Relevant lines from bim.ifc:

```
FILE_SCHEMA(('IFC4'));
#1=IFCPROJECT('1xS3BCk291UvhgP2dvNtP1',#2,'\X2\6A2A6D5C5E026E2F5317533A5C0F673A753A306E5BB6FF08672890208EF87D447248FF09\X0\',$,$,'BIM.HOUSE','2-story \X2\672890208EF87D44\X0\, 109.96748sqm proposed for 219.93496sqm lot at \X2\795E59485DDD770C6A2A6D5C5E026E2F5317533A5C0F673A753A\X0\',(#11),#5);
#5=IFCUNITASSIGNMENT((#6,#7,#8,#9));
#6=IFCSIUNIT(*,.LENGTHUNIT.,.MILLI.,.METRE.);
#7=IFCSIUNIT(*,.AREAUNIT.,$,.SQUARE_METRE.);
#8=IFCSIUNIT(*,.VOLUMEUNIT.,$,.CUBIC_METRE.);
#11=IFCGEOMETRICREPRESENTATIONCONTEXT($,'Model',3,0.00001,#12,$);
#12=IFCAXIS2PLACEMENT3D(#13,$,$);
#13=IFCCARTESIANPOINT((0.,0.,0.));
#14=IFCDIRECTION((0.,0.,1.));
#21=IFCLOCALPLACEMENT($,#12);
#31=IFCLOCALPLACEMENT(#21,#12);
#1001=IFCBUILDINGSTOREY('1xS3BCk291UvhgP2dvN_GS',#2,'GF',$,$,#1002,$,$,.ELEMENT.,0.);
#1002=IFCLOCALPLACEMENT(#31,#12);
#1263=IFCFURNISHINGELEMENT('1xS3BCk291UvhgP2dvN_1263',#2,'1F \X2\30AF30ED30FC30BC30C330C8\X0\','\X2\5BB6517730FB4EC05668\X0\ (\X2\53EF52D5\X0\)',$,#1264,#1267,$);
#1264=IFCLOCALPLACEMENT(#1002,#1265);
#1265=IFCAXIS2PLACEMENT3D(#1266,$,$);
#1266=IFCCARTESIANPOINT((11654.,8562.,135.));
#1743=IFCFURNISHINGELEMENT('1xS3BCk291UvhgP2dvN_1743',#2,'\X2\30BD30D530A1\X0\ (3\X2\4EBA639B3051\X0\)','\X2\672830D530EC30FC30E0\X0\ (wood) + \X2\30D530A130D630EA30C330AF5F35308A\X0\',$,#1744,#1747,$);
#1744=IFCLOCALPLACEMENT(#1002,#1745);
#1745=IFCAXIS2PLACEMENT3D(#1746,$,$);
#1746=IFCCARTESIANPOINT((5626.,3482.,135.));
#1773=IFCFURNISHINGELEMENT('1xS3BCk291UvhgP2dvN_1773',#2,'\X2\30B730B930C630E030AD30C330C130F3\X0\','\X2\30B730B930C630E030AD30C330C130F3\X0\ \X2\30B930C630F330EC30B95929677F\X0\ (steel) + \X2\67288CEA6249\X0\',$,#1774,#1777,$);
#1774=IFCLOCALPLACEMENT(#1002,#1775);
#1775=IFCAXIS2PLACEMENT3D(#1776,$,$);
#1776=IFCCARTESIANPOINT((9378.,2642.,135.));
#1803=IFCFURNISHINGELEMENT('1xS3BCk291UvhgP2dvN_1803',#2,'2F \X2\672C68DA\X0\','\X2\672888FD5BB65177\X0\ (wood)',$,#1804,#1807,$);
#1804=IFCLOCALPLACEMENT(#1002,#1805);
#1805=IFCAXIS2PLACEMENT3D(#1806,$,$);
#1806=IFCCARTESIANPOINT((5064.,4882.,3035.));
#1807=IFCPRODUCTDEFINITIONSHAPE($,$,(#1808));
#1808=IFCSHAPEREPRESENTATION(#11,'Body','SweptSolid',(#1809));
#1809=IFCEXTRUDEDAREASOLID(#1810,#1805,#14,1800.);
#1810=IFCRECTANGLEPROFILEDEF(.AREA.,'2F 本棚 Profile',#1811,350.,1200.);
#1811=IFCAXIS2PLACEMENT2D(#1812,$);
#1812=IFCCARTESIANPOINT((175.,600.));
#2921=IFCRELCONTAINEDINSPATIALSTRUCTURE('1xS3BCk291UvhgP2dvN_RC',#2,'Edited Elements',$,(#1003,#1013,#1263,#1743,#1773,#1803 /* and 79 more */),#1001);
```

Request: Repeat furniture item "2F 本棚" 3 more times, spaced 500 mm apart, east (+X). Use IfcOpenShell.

```python
import numpy as np
import ifcopenshell
import ifcopenshell.api.geometry
import ifcopenshell.api.root
import ifcopenshell.util.element
import ifcopenshell.util.placement

model = ifcopenshell.open("bim.ifc")


def reuse_history(source, copy):
    """copy_class also copies each property set's owner history, people and application; keep the originals."""
    for rel in copy.IsDefinedBy:
        if rel.is_a("IfcRelDefinesByProperties") and (history := rel.RelatingPropertyDefinition.OwnerHistory):
            rel.RelatingPropertyDefinition.OwnerHistory = source.OwnerHistory
            ifcopenshell.util.element.remove_deep2(model, history)


source = model.by_id(1803)
base = ifcopenshell.util.placement.get_local_placement(source.ObjectPlacement)
step = np.array([1.0, 0.0, 0.0]) * 500.0

for i in range(1, 4):
    copy = ifcopenshell.api.root.copy_class(model, product=source)
    copy.Representation = ifcopenshell.util.element.copy_deep(
        model, source.Representation, exclude=["IfcGeometricRepresentationContext", "IfcRepresentationMap"]
    )
    reuse_history(source, copy)
    matrix = base.copy()
    matrix[:3, 3] += i * step
    print("added at", matrix[:3, 3].round(3) + 0.0)
    ifcopenshell.api.geometry.edit_object_placement(model, product=copy, matrix=matrix, is_si=False)

model.write("bim_edited.ifc")
```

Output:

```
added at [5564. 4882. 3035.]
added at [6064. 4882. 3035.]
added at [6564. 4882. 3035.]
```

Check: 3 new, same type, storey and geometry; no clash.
